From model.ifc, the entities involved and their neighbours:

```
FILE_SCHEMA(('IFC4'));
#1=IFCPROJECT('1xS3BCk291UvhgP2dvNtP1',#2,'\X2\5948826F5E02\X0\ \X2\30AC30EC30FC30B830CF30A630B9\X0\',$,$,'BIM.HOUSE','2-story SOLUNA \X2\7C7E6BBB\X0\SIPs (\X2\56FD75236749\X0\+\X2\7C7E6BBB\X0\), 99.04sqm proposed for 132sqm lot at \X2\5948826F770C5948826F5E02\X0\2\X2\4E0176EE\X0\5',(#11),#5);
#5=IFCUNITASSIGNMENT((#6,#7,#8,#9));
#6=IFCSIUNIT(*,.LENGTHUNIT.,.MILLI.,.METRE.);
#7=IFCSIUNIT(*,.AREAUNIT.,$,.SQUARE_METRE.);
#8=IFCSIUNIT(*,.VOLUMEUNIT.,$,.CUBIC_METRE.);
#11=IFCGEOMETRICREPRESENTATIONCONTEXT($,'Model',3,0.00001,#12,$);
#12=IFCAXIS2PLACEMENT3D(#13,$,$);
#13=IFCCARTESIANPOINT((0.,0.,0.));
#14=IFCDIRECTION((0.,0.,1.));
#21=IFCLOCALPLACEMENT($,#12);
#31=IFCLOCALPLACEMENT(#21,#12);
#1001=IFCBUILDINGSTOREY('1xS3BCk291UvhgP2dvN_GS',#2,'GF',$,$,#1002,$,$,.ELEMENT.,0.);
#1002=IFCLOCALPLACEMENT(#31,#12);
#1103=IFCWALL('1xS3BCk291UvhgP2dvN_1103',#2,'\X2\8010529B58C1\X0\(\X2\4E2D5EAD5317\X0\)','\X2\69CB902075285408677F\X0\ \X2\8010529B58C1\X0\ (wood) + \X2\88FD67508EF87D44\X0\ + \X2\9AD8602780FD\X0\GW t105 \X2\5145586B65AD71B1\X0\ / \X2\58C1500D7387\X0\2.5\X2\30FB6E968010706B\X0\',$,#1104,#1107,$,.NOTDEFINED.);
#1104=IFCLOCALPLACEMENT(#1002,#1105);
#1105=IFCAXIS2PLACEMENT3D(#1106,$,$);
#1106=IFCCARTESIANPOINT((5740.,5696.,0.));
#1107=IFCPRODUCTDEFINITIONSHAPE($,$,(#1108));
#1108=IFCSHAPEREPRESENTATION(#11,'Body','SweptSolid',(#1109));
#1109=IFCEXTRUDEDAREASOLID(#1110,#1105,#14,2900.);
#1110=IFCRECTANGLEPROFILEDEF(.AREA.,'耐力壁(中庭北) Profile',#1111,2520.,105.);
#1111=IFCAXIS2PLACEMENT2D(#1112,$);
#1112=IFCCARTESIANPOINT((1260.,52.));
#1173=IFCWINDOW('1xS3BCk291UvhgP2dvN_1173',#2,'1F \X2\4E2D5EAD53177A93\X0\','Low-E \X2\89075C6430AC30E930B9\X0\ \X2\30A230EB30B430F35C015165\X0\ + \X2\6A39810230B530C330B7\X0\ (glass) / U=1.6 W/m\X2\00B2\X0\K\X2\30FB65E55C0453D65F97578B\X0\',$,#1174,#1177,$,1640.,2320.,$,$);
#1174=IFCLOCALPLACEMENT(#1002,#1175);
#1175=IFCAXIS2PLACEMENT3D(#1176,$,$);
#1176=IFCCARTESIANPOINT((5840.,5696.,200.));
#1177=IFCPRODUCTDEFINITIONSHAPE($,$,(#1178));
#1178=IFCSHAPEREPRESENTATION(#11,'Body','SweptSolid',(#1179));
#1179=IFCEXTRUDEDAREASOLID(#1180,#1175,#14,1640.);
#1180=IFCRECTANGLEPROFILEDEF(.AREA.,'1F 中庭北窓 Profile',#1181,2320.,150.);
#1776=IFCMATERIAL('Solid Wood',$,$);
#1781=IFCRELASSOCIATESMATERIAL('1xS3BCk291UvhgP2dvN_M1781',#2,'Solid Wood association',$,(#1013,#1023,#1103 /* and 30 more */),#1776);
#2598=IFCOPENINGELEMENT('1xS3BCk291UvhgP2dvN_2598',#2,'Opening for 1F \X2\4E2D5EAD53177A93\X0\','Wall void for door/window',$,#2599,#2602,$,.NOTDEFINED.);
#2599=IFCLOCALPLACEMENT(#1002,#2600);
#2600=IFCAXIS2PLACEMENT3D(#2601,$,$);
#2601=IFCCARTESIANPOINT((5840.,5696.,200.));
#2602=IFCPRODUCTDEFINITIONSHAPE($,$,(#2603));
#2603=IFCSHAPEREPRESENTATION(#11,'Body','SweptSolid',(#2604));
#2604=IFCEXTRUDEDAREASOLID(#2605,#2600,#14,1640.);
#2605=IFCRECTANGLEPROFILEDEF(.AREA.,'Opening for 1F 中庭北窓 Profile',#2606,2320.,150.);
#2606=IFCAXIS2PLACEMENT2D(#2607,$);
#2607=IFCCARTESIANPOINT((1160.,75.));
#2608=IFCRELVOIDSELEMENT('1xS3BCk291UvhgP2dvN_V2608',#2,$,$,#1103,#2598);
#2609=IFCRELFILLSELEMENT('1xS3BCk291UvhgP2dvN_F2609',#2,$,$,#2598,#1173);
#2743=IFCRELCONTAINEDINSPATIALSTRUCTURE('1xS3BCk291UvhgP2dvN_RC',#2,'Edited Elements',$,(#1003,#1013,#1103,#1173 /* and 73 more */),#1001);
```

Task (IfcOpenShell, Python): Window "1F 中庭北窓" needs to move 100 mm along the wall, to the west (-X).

```python
import ifcopenshell
import ifcopenshell.api.geometry
import ifcopenshell.util.placement
import ifcopenshell.util.unit

model = ifcopenshell.open("model.ifc")
unit_scale = ifcopenshell.util.unit.calculate_unit_scale(model)

window = model.by_guid("1xS3BCk291UvhgP2dvN_1173")
opening = window.FillsVoids[0].RelatingOpeningElement
wall = opening.VoidsElements[0].RelatingBuildingElement

wall_matrix = ifcopenshell.util.placement.get_local_placement(wall.ObjectPlacement)
shift = wall_matrix[:3, 0] * -0.1 / unit_scale
before = ifcopenshell.util.placement.get_local_placement(window.ObjectPlacement)[:3, 3].copy()

# The window is not placed relative to its opening, so move both.
for product in (opening, window):
    matrix = ifcopenshell.util.placement.get_local_placement(product.ObjectPlacement)
    matrix[:3, 3] += shift
    ifcopenshell.api.geometry.edit_object_placement(model, product=product, matrix=matrix, is_si=False)

after = ifcopenshell.util.placement.get_local_placement(window.ObjectPlacement)[:3, 3]
print("window moved by", (after - before).round(3) + 0.0)

model.write("model-out.ifc")
```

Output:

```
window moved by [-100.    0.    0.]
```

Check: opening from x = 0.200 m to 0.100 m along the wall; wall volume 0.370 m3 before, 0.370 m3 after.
